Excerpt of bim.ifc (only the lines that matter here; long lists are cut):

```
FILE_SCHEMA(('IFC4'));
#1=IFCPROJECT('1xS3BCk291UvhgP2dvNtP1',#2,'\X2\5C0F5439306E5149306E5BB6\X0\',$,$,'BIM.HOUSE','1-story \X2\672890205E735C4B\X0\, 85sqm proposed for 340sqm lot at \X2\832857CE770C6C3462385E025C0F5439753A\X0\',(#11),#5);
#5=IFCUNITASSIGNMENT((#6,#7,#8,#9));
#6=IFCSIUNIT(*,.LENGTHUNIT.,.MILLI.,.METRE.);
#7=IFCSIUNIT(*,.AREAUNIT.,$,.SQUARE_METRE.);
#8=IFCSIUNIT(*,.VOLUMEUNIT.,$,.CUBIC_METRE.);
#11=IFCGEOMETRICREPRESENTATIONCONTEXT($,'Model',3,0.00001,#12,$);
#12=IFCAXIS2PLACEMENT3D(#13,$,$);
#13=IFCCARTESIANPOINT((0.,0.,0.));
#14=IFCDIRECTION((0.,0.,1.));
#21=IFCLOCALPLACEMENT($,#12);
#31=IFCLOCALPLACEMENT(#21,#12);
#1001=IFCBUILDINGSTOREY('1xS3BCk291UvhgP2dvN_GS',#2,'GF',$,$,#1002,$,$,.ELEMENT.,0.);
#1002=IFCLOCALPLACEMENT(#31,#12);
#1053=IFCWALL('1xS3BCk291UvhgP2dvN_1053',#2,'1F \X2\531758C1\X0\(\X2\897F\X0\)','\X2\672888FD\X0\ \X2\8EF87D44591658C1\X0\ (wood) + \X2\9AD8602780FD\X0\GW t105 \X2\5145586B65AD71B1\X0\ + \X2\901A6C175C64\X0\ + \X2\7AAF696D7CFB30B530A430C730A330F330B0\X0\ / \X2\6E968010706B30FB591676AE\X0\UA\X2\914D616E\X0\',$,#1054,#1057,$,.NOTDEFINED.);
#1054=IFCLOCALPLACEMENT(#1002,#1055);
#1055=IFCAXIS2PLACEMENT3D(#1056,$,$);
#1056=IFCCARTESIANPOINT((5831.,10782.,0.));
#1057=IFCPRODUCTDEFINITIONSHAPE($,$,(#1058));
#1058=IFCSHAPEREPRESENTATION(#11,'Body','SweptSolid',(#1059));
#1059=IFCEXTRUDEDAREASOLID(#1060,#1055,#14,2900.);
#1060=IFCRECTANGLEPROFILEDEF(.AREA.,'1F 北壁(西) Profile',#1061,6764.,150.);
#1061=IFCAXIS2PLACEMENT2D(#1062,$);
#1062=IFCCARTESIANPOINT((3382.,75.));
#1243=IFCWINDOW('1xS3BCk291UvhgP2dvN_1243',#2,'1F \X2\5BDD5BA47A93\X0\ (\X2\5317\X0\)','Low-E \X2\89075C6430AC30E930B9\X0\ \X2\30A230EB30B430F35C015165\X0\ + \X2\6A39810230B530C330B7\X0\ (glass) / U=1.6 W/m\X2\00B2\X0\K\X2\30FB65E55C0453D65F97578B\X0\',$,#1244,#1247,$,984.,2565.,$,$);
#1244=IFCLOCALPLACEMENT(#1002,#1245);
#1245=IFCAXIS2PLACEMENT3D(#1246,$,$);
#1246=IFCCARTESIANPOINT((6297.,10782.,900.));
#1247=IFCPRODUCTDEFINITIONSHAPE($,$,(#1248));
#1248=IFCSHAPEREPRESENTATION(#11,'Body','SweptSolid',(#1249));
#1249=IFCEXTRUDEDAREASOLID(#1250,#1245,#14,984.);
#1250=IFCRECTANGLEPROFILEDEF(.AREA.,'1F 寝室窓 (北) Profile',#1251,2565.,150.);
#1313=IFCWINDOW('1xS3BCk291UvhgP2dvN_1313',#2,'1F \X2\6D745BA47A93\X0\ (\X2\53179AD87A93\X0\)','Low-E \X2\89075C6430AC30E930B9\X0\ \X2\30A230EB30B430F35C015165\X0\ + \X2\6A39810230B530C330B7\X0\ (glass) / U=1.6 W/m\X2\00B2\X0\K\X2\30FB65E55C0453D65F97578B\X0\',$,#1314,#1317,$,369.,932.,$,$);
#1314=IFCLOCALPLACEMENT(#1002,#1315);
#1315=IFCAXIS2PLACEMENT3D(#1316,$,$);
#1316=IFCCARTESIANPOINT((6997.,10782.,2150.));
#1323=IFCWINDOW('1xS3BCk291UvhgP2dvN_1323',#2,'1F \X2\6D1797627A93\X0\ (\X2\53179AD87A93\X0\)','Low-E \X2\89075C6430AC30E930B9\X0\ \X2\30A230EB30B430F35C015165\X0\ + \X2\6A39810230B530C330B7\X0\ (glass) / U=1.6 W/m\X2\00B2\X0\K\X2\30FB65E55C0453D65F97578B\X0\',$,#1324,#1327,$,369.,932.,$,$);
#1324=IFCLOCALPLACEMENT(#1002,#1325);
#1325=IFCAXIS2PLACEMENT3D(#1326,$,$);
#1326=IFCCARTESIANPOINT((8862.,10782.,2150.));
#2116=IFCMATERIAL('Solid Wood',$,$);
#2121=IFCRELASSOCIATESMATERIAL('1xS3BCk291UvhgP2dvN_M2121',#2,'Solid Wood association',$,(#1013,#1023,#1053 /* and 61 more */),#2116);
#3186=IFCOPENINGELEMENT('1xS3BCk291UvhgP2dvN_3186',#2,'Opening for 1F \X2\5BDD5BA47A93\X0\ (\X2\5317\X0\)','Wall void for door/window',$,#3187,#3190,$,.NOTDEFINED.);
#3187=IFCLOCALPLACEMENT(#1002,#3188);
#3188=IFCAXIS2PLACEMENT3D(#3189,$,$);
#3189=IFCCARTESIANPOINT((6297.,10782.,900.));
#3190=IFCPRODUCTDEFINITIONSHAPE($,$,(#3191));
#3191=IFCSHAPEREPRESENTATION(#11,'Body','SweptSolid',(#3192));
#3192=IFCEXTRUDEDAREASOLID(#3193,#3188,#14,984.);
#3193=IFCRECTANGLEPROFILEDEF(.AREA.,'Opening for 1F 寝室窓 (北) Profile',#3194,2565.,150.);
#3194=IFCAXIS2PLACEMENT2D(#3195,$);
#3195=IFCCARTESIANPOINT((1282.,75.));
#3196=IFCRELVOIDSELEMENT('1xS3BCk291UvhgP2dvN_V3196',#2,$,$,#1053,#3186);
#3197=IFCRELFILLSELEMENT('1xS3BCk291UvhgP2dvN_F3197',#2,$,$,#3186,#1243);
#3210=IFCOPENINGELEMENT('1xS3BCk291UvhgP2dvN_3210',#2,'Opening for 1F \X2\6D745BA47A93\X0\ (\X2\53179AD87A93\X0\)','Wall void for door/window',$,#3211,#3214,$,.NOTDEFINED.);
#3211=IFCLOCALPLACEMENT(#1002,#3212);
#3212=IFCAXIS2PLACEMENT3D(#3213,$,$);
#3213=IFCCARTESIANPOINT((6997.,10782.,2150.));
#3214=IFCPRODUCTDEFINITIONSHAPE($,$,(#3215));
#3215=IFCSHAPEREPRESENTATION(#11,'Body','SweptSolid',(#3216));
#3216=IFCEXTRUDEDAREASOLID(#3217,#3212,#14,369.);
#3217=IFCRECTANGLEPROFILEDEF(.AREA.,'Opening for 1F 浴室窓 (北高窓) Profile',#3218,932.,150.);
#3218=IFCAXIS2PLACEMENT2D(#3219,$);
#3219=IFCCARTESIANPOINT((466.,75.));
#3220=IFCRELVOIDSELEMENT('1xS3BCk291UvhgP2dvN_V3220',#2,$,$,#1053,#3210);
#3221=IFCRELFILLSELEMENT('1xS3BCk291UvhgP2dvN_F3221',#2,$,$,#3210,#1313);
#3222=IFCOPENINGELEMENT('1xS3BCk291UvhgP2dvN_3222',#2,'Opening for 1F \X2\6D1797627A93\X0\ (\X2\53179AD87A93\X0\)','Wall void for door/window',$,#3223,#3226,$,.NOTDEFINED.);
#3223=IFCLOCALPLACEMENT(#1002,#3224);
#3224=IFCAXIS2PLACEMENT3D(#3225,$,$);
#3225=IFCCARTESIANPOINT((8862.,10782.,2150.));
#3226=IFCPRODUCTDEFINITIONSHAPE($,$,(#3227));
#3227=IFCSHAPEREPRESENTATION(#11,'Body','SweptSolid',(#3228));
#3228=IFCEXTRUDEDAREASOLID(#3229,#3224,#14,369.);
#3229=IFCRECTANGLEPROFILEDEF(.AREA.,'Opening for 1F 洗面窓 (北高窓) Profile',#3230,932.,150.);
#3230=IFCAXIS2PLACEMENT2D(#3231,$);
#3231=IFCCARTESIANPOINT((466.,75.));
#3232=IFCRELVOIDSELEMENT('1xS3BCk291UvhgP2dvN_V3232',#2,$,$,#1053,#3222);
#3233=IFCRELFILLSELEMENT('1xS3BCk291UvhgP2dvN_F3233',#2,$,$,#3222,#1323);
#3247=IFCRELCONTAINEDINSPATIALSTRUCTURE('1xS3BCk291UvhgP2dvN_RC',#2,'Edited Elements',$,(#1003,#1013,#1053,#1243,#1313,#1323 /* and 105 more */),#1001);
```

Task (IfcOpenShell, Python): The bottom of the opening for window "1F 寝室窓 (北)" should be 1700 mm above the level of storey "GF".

```python
import numpy as np
import ifcopenshell
import ifcopenshell.api.geometry
import ifcopenshell.geom
import ifcopenshell.util.element
import ifcopenshell.util.placement
import ifcopenshell.util.shape
import ifcopenshell.util.unit

model = ifcopenshell.open("bim.ifc")
unit_scale = ifcopenshell.util.unit.calculate_unit_scale(model)

window = model.by_guid("1xS3BCk291UvhgP2dvN_1243")
opening = window.FillsVoids[0].RelatingOpeningElement
storey = ifcopenshell.util.element.get_container(window, ifc_class="IfcBuildingStorey")
level = ifcopenshell.util.placement.get_local_placement(storey.ObjectPlacement)[2, 3]

# The opening's origin need not be at the sill, so measure its lowest point.
shape = ifcopenshell.geom.create_shape(ifcopenshell.geom.settings(), opening)
bottom = ifcopenshell.util.shape.get_shape_bottom_elevation(shape, shape.geometry) / unit_scale
dz = level + 1700.0 - bottom

shift = np.array([0.0, 0.0, dz])
# The window is not placed relative to its opening, so move both.
for product in (opening, window):
    matrix = ifcopenshell.util.placement.get_local_placement(product.ObjectPlacement)
    matrix[:3, 3] += shift
    ifcopenshell.api.geometry.edit_object_placement(model, product=product, matrix=matrix, is_si=False)

print(f"moved by {dz * unit_scale:+.3f} m")

model.write("bim_rev.ifc")
```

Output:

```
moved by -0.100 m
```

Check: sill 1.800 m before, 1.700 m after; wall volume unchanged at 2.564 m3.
